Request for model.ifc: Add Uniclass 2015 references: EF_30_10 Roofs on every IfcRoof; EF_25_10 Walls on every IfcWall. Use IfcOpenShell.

First a look at what the model holds.

```python
import ifcopenshell

model = ifcopenshell.open("model.ifc")
print(model.schema)
print("classifications:", [c.Name for c in model.by_type("IfcClassification")])
for ifc_class in ("IfcDoor", "IfcRoof", "IfcStair", "IfcWall", "IfcWindow"):
    print(ifc_class, len(model.by_type(ifc_class)))
```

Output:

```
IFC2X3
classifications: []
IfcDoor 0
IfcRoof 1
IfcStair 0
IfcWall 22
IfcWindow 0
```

```python
import ifcopenshell
import ifcopenshell.api.classification

model = ifcopenshell.open("model.ifc")

# IFC2X3 requires Source and Edition and has no link from the project to the system.
system = model.create_entity("IfcClassification", Source="NBS", Edition="2015", Name="Uniclass 2015")

codes = {
    "IfcRoof": ("EF_30_10", "Roofs"),
    "IfcWall": ("EF_25_10", "Walls"),
}
for ifc_class, (code, name) in codes.items():
    products = model.by_type(ifc_class)
    ifcopenshell.api.classification.add_reference(
        model, products=products, classification=system, identification=code, name=name
    )
    print(code, len(products))

model.write("model_updated.ifc")
```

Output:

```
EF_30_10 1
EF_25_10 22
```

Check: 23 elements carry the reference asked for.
